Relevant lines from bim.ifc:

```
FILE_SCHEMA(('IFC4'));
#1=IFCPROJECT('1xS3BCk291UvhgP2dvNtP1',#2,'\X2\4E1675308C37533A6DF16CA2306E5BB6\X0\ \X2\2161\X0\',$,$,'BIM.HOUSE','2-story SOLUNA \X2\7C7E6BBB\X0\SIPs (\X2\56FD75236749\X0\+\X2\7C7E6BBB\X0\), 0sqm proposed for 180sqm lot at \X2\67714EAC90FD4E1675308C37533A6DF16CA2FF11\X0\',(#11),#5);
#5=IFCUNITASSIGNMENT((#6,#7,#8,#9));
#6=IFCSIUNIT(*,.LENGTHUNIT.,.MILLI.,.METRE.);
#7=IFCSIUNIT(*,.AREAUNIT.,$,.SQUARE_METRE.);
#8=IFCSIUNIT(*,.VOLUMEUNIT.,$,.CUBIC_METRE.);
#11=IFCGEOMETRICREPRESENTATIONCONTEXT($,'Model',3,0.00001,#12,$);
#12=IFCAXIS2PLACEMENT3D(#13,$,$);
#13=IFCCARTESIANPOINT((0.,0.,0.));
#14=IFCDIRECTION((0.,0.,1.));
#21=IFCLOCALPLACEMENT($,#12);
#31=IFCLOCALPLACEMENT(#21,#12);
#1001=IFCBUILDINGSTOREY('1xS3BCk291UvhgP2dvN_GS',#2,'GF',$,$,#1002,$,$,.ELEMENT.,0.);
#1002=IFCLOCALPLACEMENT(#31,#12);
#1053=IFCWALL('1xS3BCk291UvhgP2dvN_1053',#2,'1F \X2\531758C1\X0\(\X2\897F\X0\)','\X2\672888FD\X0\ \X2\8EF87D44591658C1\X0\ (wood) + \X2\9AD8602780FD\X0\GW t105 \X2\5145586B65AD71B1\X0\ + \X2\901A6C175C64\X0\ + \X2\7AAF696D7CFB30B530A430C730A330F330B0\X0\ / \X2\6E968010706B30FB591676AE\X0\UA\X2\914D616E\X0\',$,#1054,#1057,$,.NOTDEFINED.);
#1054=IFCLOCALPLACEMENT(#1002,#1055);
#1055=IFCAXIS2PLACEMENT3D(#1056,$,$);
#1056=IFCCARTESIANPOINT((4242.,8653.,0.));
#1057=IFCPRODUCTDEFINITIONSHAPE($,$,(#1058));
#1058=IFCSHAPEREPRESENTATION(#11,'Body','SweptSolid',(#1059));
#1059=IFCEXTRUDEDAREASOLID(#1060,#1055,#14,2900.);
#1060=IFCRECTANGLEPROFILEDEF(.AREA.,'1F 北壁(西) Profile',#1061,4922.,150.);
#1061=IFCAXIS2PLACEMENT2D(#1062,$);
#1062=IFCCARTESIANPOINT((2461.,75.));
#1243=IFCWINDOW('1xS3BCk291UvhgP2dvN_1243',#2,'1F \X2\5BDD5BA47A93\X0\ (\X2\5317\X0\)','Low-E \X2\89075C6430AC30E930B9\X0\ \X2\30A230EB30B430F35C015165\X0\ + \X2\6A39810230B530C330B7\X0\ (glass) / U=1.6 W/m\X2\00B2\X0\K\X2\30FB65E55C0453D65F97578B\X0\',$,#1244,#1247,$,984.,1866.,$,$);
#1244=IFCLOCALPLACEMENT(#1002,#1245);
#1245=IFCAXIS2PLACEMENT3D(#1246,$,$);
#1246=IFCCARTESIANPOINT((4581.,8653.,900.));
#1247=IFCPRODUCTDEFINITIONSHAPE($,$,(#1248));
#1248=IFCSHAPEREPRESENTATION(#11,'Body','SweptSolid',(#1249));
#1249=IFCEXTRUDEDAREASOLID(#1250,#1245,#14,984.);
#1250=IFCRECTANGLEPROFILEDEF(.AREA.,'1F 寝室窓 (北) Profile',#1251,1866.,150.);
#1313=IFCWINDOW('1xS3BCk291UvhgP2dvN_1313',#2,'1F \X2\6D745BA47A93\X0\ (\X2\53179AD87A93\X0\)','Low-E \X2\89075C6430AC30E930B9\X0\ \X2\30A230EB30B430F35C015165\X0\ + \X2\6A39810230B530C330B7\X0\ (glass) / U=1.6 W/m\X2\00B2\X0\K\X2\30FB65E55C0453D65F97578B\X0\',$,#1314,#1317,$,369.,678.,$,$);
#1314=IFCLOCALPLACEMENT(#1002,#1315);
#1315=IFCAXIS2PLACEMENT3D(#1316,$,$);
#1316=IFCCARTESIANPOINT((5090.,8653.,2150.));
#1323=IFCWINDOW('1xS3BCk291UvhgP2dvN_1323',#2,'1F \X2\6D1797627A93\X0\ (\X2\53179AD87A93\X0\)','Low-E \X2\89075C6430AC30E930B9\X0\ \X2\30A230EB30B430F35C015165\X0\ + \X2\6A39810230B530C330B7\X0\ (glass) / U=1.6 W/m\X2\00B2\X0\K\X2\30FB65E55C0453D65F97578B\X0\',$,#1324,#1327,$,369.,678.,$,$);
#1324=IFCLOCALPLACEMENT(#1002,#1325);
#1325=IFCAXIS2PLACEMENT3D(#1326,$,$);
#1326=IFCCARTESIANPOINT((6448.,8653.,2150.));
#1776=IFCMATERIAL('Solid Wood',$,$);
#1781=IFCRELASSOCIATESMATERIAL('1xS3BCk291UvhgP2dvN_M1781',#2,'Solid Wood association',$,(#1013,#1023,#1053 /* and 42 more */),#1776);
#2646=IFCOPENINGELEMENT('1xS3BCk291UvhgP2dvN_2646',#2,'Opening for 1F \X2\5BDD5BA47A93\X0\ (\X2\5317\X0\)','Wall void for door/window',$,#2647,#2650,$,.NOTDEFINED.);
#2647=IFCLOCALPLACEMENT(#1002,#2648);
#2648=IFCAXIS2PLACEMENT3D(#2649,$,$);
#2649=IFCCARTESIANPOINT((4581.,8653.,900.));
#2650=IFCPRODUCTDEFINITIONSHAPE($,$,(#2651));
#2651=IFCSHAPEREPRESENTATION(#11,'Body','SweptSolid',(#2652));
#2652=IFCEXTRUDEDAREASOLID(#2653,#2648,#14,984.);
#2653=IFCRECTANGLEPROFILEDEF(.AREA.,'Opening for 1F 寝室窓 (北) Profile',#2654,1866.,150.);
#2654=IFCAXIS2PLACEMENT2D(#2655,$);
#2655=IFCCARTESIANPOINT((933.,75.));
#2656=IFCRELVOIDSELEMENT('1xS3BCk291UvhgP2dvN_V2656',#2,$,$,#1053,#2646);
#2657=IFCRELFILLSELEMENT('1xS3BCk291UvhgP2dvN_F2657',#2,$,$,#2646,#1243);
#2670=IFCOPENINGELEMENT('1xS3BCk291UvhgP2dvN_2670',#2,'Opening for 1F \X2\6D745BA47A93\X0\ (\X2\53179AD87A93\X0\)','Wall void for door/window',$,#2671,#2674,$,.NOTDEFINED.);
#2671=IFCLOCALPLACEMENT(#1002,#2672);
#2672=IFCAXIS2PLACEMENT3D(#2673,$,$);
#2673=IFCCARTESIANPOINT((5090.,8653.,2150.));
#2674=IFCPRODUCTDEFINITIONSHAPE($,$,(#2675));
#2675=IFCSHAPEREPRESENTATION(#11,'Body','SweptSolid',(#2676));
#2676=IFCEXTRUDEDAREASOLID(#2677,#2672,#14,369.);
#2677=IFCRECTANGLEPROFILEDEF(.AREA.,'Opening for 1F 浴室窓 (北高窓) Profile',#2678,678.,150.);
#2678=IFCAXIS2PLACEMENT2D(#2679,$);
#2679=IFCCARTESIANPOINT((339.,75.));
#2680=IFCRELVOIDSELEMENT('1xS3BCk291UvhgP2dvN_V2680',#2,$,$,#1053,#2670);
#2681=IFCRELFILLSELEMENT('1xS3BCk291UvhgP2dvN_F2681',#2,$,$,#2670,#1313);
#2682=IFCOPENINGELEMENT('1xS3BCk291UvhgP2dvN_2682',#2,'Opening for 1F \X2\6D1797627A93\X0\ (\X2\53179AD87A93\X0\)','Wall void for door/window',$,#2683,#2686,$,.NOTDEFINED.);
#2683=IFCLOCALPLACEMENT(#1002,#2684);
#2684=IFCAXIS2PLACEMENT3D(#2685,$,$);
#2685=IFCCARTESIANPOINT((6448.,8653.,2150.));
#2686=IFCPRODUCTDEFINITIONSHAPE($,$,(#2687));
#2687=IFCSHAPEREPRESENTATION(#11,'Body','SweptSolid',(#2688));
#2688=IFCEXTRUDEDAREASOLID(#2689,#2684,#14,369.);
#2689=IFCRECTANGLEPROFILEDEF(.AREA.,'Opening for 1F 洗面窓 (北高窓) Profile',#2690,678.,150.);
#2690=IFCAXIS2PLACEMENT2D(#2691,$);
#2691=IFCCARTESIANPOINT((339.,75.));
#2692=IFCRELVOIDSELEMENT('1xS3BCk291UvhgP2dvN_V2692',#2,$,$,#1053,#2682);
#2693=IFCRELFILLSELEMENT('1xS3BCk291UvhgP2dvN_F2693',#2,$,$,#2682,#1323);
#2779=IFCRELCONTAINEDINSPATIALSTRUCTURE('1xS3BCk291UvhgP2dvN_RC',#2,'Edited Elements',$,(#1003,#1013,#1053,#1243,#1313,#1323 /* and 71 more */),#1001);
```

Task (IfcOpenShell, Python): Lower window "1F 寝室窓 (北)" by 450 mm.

```python
import numpy as np
import ifcopenshell
import ifcopenshell.api.geometry
import ifcopenshell.util.placement
import ifcopenshell.util.unit

model = ifcopenshell.open("bim.ifc")
unit_scale = ifcopenshell.util.unit.calculate_unit_scale(model)

window = model.by_id(1243)
opening = window.FillsVoids[0].RelatingOpeningElement
dz = -0.45 / unit_scale

shift = np.array([0.0, 0.0, dz])
# The window is not placed relative to its opening, so move both.
for product in (opening, window):
    matrix = ifcopenshell.util.placement.get_local_placement(product.ObjectPlacement)
    matrix[:3, 3] += shift
    ifcopenshell.api.geometry.edit_object_placement(model, product=product, matrix=matrix, is_si=False)

print(f"moved by {dz * unit_scale:+.3f} m")

model.write("bim_v2.ifc")
```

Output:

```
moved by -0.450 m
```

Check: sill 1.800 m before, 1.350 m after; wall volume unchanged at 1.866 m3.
